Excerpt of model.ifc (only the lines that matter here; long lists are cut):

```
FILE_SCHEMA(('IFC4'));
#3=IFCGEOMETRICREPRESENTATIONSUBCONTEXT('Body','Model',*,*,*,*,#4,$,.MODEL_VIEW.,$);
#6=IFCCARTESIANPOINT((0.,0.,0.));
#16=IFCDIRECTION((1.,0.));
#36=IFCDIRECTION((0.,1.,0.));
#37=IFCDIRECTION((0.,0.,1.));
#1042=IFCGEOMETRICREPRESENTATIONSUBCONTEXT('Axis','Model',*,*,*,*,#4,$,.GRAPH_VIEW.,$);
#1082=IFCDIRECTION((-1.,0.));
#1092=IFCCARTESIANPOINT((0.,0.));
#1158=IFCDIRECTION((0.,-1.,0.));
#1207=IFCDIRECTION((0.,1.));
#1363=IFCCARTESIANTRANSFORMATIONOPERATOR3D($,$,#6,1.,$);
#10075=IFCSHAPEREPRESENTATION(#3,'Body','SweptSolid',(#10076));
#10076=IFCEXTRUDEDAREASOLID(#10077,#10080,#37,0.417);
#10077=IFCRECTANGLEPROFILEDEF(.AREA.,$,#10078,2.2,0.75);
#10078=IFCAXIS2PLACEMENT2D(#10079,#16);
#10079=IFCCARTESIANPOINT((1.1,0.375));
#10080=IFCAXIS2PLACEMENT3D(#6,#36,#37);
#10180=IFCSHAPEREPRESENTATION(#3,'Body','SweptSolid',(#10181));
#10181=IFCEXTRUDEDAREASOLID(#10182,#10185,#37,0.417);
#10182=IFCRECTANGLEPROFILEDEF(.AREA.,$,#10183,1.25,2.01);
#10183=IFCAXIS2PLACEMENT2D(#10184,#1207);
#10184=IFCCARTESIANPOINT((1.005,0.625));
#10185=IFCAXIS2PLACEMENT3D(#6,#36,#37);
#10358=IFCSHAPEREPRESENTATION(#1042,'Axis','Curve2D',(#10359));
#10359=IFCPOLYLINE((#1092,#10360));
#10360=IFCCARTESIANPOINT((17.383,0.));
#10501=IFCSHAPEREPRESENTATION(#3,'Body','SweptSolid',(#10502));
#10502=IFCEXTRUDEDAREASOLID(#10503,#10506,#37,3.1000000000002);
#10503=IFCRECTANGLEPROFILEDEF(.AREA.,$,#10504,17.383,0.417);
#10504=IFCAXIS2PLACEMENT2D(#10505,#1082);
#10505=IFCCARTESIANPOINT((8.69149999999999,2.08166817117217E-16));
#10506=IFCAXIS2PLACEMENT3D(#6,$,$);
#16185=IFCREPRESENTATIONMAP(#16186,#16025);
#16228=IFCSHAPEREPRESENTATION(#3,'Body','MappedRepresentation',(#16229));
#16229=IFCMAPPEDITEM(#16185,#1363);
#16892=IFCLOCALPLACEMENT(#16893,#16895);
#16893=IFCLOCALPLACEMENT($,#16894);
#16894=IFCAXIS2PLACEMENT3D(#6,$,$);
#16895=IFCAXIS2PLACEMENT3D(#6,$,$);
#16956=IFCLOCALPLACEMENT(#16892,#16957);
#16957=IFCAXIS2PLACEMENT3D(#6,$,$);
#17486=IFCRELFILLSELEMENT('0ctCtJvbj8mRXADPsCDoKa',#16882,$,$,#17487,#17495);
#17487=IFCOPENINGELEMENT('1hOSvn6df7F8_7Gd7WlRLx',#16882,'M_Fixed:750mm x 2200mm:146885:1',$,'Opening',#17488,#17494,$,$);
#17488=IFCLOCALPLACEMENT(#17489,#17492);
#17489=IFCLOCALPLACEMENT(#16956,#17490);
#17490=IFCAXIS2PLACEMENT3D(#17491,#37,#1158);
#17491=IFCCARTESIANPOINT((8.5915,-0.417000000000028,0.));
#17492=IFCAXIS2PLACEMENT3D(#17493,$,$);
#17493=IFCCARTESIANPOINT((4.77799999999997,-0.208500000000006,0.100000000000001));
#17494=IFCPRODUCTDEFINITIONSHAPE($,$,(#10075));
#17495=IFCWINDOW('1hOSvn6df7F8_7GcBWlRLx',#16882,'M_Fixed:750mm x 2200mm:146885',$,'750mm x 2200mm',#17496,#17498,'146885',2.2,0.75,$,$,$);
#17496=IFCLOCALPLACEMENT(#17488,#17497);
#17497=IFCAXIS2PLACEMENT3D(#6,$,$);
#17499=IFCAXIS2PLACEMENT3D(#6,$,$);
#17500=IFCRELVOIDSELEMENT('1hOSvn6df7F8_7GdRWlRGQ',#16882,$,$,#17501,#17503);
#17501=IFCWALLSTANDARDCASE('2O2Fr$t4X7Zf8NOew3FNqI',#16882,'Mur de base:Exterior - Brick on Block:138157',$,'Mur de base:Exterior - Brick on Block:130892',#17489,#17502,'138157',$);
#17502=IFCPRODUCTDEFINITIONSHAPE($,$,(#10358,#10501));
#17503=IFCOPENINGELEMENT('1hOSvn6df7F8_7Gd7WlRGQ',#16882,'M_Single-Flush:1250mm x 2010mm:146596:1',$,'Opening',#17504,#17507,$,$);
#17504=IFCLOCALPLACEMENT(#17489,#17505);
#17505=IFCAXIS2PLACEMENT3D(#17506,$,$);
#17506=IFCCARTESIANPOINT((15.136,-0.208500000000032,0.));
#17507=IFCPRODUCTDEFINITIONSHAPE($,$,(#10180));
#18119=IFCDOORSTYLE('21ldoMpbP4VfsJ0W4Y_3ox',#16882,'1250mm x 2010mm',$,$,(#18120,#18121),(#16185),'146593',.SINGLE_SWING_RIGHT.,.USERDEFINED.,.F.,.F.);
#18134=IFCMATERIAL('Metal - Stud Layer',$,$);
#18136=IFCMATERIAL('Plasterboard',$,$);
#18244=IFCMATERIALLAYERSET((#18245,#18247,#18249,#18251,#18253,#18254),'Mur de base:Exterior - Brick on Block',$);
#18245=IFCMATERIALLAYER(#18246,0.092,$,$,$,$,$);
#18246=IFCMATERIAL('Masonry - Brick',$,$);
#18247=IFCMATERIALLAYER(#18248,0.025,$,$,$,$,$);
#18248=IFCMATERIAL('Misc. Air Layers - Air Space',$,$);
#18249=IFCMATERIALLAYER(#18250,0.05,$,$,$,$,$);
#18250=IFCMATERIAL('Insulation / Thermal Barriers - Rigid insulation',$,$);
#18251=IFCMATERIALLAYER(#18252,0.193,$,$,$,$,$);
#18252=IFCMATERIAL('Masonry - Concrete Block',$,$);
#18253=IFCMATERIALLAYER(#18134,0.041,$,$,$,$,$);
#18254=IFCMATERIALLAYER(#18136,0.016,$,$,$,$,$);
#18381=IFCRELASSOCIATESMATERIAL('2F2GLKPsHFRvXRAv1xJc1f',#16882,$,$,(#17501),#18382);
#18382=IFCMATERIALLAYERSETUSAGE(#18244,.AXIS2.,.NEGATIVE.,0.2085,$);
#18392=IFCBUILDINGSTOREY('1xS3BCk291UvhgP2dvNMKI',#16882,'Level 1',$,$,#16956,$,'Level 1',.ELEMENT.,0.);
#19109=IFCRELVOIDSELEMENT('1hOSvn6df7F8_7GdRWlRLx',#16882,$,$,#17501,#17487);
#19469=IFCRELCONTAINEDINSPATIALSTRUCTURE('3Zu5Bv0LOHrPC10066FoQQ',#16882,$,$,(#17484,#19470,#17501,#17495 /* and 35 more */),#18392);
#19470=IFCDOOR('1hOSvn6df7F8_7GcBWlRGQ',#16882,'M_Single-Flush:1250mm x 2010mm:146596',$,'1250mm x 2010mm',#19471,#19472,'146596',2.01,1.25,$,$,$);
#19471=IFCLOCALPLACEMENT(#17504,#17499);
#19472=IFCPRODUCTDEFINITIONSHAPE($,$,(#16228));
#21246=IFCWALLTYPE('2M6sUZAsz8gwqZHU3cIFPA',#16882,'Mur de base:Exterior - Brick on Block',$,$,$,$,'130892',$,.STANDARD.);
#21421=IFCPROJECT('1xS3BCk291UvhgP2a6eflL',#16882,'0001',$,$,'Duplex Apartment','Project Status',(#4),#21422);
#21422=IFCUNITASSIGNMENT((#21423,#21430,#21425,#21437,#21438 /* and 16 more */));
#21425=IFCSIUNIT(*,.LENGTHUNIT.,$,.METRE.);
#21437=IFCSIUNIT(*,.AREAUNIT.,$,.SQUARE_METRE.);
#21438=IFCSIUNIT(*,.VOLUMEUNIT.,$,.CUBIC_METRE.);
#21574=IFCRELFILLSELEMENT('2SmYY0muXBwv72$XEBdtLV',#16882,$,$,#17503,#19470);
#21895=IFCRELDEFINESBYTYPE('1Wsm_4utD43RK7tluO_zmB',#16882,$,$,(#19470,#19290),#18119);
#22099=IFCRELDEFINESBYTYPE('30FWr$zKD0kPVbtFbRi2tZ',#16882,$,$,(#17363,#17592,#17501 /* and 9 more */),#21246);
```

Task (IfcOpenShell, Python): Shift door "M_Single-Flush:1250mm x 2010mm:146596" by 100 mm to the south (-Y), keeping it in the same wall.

```python
import ifcopenshell
import ifcopenshell.api.geometry
import ifcopenshell.util.placement

model = ifcopenshell.open("model.ifc")

door = model.by_guid("1hOSvn6df7F8_7GcBWlRGQ")
opening = door.FillsVoids[0].RelatingOpeningElement
wall = opening.VoidsElements[0].RelatingBuildingElement

wall_matrix = ifcopenshell.util.placement.get_local_placement(wall.ObjectPlacement)
shift = wall_matrix[:3, 0] * 0.1
before = ifcopenshell.util.placement.get_local_placement(door.ObjectPlacement)[:3, 3].copy()

# The door is placed relative to its opening, so it follows when the opening moves.
matrix = ifcopenshell.util.placement.get_local_placement(opening.ObjectPlacement)
matrix[:3, 3] += shift
ifcopenshell.api.geometry.edit_object_placement(
    model, product=opening, matrix=matrix, is_si=False, should_transform_children=True
)

after = ifcopenshell.util.placement.get_local_placement(door.ObjectPlacement)[:3, 3]
print("door moved by", (after - before).round(3) + 0.0)

model.write("model_updated.ifc")
```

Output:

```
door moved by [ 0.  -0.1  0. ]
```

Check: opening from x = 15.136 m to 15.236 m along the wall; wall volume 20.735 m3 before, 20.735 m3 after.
